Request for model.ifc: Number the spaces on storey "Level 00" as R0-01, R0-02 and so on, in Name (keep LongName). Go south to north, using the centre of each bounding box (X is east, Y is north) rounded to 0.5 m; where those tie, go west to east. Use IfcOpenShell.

First a look at what the model holds.

```python
import ifcopenshell
import ifcopenshell.util.element
import ifcopenshell.util.placement

model = ifcopenshell.open("model.ifc")
print(model.schema)
storey = next(s for s in model.by_type("IfcBuildingStorey") if s.Name == "Level 00")
spaces = [e for e in ifcopenshell.util.element.get_decomposition(storey) if e.is_a("IfcSpace")]
for e in sorted(spaces, key=lambda e: e.id()):
    origin = ifcopenshell.util.placement.get_local_placement(e.ObjectPlacement)[:3, 3]
    print(e.id(), e.Name, e.LongName, origin.round(2) + 0.0, sep=" | ")
```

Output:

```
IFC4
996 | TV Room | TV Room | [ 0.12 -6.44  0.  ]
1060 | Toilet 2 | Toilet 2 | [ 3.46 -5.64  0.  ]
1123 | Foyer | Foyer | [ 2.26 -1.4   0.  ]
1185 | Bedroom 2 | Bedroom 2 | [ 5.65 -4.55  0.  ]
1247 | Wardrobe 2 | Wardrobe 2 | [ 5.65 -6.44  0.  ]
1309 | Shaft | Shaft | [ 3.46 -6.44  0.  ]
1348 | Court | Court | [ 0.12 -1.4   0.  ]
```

```python
import ifcopenshell
import ifcopenshell.geom
import ifcopenshell.util.element
import ifcopenshell.util.shape

model = ifcopenshell.open("model.ifc")
settings = ifcopenshell.geom.settings()
settings.set("use-world-coords", True)


def centre(element):
    shape = ifcopenshell.geom.create_shape(settings, element)
    return ifcopenshell.util.shape.get_bbox_centroid(shape.geometry)


storey = next(s for s in model.by_type("IfcBuildingStorey") if s.Name == "Level 00")
spaces = [e for e in ifcopenshell.util.element.get_decomposition(storey) if e.is_a("IfcSpace")]

# Insertion points can sit at a corner or the storey origin, so sort by the geometry (in metres).
centres = {e: centre(e) for e in spaces}
spaces.sort(key=lambda e: (round(centres[e][1] / 0.5), centres[e][0]))

for i, e in enumerate(spaces, start=1):
    number = f"R0-{i:02d}"
    e.Name = number
    print(e.id(), number)

model.write("model-out.ifc")
```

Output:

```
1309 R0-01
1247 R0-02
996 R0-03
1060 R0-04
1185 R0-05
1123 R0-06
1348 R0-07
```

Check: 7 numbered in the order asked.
